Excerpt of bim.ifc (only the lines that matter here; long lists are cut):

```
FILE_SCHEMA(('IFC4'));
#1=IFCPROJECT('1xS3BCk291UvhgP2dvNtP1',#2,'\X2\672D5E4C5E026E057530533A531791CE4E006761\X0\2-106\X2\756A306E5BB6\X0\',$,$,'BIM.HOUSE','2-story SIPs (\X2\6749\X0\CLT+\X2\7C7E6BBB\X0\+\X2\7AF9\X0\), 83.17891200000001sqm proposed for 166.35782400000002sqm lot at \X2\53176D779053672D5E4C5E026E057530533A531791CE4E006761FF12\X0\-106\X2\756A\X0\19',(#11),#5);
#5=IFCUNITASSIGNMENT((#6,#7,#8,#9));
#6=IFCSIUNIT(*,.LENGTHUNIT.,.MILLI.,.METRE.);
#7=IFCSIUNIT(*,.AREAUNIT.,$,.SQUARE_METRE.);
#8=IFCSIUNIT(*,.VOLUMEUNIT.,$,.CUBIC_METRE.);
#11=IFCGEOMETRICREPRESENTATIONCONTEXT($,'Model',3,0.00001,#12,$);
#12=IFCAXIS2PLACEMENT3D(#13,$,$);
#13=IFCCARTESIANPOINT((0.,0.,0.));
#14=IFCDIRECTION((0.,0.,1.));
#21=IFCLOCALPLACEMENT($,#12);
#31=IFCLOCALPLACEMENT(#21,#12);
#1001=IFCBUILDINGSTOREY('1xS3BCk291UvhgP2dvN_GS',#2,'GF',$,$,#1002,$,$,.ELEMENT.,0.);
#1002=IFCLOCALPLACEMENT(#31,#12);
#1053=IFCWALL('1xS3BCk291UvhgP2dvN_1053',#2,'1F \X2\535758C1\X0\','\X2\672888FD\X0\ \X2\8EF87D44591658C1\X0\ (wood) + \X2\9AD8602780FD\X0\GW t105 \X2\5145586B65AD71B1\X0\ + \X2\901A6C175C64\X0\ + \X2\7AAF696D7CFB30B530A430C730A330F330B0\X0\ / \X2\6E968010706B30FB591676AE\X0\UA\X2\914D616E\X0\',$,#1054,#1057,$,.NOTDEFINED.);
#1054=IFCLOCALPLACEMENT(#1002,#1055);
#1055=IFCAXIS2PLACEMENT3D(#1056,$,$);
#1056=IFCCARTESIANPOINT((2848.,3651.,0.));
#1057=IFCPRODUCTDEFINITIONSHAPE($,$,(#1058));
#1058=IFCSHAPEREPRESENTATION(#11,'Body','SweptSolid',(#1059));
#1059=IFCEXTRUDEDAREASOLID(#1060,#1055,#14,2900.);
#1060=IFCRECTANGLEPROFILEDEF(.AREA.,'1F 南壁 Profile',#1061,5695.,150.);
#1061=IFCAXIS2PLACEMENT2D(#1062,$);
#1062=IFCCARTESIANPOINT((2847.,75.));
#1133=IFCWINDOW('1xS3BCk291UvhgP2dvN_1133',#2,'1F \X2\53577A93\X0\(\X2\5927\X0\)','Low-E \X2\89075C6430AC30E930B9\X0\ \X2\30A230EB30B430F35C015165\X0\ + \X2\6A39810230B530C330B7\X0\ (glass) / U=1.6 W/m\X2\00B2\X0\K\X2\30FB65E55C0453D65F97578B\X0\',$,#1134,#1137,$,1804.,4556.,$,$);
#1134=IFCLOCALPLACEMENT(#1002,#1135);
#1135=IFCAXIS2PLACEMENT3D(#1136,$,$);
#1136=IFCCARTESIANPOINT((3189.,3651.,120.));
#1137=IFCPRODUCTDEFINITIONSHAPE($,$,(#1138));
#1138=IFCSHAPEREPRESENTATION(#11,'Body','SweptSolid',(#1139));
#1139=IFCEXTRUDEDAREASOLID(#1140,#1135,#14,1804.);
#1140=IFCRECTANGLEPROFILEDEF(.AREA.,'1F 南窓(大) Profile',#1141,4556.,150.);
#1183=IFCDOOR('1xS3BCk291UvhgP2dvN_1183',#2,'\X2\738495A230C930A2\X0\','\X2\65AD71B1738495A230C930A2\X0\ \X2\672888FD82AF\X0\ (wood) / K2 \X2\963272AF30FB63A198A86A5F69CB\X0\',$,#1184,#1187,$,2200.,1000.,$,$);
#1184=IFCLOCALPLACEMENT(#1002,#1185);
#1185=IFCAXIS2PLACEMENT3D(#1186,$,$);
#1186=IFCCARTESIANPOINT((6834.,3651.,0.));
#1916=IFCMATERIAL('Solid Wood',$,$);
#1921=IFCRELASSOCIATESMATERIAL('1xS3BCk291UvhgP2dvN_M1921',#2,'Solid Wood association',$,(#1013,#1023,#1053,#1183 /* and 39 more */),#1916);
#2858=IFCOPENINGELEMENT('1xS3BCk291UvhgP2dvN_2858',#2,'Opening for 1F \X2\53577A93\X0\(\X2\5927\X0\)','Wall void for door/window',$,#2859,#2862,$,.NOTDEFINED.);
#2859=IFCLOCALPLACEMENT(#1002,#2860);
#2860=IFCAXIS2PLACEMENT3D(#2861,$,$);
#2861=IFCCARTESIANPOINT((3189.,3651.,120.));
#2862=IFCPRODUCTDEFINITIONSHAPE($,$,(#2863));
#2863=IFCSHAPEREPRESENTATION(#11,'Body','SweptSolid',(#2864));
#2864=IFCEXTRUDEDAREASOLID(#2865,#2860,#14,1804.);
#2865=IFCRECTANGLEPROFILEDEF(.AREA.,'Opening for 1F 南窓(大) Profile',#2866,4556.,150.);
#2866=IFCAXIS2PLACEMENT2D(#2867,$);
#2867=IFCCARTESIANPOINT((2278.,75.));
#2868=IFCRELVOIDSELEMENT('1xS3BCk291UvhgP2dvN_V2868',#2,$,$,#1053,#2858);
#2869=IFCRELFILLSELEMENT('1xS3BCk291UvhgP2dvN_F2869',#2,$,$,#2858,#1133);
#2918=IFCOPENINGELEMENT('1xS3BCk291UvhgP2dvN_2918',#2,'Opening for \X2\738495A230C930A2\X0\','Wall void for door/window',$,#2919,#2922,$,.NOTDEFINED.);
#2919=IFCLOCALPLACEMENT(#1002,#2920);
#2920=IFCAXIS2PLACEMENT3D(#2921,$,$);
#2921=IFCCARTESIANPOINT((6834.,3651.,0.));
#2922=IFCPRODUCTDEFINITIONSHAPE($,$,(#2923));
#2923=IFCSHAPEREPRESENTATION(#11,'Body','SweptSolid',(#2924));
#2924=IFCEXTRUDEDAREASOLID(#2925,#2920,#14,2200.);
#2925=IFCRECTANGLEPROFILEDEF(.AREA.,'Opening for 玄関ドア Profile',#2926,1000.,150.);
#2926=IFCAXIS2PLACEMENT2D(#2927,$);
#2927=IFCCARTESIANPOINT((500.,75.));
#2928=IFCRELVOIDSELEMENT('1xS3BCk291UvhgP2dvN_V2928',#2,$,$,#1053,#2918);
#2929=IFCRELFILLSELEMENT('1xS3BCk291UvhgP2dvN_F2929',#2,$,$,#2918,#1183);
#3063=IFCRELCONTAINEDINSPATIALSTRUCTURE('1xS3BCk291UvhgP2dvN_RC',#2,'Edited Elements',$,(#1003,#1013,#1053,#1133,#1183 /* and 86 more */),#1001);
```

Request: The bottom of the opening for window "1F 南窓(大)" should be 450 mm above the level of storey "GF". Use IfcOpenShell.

```python
import numpy as np
import ifcopenshell
import ifcopenshell.api.geometry
import ifcopenshell.geom
import ifcopenshell.util.element
import ifcopenshell.util.placement
import ifcopenshell.util.shape
import ifcopenshell.util.unit

model = ifcopenshell.open("bim.ifc")
unit_scale = ifcopenshell.util.unit.calculate_unit_scale(model)

window = model.by_id(1133)
opening = window.FillsVoids[0].RelatingOpeningElement
storey = ifcopenshell.util.element.get_container(window, ifc_class="IfcBuildingStorey")
level = ifcopenshell.util.placement.get_local_placement(storey.ObjectPlacement)[2, 3]

# The opening's origin need not be at the sill, so measure its lowest point.
shape = ifcopenshell.geom.create_shape(ifcopenshell.geom.settings(), opening)
bottom = ifcopenshell.util.shape.get_shape_bottom_elevation(shape, shape.geometry) / unit_scale
dz = level + 450.0 - bottom

shift = np.array([0.0, 0.0, dz])
# The window is not placed relative to its opening, so move both.
for product in (opening, window):
    matrix = ifcopenshell.util.placement.get_local_placement(product.ObjectPlacement)
    matrix[:3, 3] += shift
    ifcopenshell.api.geometry.edit_object_placement(model, product=product, matrix=matrix, is_si=False)

print(f"moved by {dz * unit_scale:+.3f} m")

model.write("bim_updated.ifc")
```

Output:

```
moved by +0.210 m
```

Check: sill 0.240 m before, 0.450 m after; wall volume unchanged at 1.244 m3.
